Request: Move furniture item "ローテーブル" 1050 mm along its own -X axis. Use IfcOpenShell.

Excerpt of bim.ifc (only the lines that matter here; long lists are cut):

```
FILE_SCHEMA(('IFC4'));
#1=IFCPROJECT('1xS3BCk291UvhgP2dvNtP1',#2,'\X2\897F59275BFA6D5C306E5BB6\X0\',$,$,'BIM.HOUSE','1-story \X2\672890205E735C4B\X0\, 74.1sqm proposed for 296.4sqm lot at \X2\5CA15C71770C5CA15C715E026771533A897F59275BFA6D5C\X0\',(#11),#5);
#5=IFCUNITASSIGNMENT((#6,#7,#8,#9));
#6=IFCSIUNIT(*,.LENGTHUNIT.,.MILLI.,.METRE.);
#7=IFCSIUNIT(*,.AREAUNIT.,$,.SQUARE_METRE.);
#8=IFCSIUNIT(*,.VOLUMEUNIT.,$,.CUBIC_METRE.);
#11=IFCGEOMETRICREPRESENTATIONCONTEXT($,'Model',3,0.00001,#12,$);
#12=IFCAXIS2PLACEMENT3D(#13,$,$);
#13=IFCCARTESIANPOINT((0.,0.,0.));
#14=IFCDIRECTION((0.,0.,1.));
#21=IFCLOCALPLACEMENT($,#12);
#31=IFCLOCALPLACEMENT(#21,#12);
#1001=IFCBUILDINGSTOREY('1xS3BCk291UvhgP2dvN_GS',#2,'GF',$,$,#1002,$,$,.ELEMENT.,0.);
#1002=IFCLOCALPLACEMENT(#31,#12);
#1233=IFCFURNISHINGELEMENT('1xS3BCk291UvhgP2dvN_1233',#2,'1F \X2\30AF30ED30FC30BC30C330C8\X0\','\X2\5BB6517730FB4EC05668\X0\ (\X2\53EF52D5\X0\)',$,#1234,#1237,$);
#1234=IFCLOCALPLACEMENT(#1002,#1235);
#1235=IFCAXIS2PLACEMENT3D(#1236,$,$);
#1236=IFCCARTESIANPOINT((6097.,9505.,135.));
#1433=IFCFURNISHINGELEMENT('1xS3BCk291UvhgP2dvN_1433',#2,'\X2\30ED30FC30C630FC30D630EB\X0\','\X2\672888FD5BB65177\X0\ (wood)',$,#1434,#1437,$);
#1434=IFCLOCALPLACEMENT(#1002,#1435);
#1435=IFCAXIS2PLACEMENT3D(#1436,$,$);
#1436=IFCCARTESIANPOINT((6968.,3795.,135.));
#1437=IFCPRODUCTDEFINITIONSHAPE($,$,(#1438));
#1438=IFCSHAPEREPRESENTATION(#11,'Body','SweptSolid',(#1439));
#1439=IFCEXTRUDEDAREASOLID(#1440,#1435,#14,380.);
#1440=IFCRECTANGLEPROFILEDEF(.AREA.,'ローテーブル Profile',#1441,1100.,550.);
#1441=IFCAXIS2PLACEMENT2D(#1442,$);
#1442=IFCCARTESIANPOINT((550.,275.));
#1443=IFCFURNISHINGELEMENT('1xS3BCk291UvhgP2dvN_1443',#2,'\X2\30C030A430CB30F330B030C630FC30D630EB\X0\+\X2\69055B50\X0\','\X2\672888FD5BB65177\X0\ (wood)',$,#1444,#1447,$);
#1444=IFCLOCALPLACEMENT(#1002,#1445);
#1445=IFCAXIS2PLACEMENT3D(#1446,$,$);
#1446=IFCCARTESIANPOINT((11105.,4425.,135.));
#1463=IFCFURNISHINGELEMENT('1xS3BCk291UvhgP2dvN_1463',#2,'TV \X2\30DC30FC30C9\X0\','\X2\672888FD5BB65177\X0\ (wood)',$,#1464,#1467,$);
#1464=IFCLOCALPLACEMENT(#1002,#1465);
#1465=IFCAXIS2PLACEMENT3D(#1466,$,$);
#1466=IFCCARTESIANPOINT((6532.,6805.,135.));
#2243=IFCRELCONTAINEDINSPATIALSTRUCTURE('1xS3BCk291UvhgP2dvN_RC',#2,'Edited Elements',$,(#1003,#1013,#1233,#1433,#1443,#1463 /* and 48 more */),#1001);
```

```python
import ifcopenshell
import ifcopenshell.api.geometry
import ifcopenshell.util.placement
import ifcopenshell.util.unit

model = ifcopenshell.open("bim.ifc")
unit_scale = ifcopenshell.util.unit.calculate_unit_scale(model)

item = model.by_guid("1xS3BCk291UvhgP2dvN_1433")
matrix = ifcopenshell.util.placement.get_local_placement(item.ObjectPlacement)
matrix[:3, 3] -= matrix[:3, 0] * 1.05 / unit_scale
ifcopenshell.api.geometry.edit_object_placement(model, product=item, matrix=matrix, is_si=False)

print(ifcopenshell.util.placement.get_local_placement(item.ObjectPlacement).round(3) + 0.0)

model.write("bim-out.ifc")
```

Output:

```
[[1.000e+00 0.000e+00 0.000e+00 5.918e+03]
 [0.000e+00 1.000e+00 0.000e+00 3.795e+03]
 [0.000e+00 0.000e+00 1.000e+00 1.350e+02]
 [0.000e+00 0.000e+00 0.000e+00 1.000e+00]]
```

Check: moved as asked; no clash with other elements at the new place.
